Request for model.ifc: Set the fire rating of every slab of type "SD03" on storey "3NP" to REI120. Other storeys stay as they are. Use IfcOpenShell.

First a look at what the model holds.

```python
import ifcopenshell
import ifcopenshell.util.element

model = ifcopenshell.open("model.ifc")
print(model.schema)
storey = next(s for s in model.by_type("IfcBuildingStorey") if s.Name == "3NP")
slabs = [e for e in ifcopenshell.util.element.get_decomposition(storey) if e.is_a("IfcSlab")]
seen = {}
for e in slabs:
    element_type = ifcopenshell.util.element.get_type(e)
    key = (element_type.Name if element_type != e and element_type else None, ifcopenshell.util.element.get_pset(e, "Pset_SlabCommon", "FireRating"))
    seen[key] = seen.get(key, 0) + 1
for (name, value), count in sorted(seen.items(), key=str):
    print(count, "x", name, "|", value)
```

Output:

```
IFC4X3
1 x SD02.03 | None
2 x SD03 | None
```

```python
import ifcopenshell
import ifcopenshell.api.pset
import ifcopenshell.util.element

model = ifcopenshell.open("model.ifc")

storey = next(s for s in model.by_type("IfcBuildingStorey") if s.Name == "3NP")
slabs = [e for e in ifcopenshell.util.element.get_decomposition(storey) if e.is_a("IfcSlab")]

count = 0
for e in slabs:
    element_type = ifcopenshell.util.element.get_type(e)
    if element_type in (None, e) or element_type.Name != "SD03":
        continue
    # add_pset returns the element's existing set when there is one.
    pset = ifcopenshell.api.pset.add_pset(model, product=e, name="Pset_SlabCommon")
    ifcopenshell.api.pset.edit_pset(model, pset=pset, properties={"FireRating": "REI120"})
    count += 1

print(count, "slabs updated")

model.write("model_updated.ifc")
```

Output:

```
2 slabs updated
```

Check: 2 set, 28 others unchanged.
